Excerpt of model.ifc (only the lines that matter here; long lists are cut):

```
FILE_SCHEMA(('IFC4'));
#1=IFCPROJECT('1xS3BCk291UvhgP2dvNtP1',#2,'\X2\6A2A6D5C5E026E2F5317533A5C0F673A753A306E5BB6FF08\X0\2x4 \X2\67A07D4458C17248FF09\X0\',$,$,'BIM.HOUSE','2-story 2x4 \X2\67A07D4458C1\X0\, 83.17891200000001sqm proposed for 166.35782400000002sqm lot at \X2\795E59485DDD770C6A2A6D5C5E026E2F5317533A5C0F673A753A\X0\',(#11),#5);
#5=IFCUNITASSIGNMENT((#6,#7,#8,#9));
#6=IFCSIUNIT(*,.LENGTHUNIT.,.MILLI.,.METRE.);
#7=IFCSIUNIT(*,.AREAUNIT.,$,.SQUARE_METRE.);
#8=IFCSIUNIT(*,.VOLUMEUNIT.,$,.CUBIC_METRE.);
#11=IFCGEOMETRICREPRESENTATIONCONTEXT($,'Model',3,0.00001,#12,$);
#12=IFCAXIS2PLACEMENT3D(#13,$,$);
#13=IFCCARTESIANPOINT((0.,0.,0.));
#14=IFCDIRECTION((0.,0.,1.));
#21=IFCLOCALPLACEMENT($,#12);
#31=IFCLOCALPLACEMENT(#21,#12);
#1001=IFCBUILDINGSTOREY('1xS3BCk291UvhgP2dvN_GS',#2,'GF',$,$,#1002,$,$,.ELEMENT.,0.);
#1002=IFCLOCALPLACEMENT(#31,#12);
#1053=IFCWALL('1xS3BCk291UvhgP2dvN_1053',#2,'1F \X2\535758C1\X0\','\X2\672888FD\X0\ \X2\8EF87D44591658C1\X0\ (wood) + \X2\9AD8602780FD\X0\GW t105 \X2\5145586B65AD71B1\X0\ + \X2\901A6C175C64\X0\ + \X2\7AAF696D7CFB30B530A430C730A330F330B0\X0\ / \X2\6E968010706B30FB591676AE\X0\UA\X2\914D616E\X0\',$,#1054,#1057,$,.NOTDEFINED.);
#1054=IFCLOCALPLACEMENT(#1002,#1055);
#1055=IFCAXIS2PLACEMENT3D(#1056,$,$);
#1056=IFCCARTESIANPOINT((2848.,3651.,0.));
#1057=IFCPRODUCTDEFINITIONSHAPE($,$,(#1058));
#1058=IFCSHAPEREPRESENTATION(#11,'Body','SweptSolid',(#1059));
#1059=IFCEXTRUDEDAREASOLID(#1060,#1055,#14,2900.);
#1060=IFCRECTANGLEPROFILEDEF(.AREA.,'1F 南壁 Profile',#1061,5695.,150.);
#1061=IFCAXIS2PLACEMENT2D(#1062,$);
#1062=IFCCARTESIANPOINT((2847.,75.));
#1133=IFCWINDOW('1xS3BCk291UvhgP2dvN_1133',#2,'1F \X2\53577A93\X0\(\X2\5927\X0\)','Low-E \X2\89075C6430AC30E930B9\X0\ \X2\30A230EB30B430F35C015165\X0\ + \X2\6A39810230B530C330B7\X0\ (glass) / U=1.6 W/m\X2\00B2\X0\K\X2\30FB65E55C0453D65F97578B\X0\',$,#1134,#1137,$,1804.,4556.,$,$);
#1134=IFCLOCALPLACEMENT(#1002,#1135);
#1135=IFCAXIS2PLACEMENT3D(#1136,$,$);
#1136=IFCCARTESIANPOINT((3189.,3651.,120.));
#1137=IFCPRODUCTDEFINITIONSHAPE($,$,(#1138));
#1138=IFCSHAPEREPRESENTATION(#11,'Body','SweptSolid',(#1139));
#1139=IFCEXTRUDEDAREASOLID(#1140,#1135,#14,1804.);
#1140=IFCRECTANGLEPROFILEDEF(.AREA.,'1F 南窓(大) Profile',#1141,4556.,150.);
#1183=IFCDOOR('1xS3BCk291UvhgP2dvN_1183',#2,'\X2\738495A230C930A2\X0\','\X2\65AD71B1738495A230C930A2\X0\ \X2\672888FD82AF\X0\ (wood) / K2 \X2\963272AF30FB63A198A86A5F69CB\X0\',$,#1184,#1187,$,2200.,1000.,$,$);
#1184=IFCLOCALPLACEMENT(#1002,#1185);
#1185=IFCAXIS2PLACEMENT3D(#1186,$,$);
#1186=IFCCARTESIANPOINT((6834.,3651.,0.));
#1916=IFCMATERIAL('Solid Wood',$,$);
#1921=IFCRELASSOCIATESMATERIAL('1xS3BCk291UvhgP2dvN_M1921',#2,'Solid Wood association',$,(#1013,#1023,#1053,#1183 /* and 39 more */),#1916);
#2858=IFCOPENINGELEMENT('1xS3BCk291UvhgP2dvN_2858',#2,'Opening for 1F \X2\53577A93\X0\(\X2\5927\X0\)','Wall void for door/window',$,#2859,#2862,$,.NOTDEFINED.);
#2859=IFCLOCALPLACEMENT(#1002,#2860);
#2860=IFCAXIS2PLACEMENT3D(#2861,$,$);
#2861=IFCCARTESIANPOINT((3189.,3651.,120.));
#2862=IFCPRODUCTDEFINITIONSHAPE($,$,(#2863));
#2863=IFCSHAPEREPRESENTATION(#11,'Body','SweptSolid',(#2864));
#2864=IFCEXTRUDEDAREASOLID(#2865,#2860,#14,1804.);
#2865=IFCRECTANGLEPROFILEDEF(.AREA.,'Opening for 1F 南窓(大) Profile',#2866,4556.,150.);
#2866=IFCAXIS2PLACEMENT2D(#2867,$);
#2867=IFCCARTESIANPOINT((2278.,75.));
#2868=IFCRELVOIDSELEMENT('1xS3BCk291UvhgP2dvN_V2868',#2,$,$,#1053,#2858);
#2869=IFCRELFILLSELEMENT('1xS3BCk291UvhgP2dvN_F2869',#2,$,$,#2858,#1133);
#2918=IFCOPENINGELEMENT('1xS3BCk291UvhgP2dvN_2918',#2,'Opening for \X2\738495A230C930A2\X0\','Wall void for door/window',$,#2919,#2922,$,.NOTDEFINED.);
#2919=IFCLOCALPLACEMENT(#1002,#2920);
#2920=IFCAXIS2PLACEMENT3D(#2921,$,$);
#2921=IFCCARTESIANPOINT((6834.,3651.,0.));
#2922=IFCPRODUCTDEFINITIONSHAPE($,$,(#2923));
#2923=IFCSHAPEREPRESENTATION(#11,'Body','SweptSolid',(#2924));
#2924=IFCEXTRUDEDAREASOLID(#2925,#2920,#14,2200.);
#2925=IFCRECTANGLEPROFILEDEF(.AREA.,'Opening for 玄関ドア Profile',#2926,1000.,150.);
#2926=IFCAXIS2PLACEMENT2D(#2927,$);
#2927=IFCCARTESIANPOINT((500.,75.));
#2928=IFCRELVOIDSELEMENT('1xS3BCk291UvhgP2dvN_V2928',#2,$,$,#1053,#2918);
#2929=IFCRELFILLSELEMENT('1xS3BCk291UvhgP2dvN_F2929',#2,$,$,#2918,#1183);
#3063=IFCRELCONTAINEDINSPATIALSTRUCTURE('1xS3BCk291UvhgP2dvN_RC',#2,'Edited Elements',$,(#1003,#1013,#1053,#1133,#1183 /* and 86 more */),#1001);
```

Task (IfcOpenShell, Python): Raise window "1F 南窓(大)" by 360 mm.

```python
import numpy as np
import ifcopenshell
import ifcopenshell.api.geometry
import ifcopenshell.util.placement
import ifcopenshell.util.unit

model = ifcopenshell.open("model.ifc")
unit_scale = ifcopenshell.util.unit.calculate_unit_scale(model)

window = model.by_id(1133)
opening = window.FillsVoids[0].RelatingOpeningElement
dz = 360.0

shift = np.array([0.0, 0.0, dz])
# The window is not placed relative to its opening, so move both.
for product in (opening, window):
    matrix = ifcopenshell.util.placement.get_local_placement(product.ObjectPlacement)
    matrix[:3, 3] += shift
    ifcopenshell.api.geometry.edit_object_placement(model, product=product, matrix=matrix, is_si=False)

print(f"moved by {dz * unit_scale:+.3f} m")

model.write("model_edited.ifc")
```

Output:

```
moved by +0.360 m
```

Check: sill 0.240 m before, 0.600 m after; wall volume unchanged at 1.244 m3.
